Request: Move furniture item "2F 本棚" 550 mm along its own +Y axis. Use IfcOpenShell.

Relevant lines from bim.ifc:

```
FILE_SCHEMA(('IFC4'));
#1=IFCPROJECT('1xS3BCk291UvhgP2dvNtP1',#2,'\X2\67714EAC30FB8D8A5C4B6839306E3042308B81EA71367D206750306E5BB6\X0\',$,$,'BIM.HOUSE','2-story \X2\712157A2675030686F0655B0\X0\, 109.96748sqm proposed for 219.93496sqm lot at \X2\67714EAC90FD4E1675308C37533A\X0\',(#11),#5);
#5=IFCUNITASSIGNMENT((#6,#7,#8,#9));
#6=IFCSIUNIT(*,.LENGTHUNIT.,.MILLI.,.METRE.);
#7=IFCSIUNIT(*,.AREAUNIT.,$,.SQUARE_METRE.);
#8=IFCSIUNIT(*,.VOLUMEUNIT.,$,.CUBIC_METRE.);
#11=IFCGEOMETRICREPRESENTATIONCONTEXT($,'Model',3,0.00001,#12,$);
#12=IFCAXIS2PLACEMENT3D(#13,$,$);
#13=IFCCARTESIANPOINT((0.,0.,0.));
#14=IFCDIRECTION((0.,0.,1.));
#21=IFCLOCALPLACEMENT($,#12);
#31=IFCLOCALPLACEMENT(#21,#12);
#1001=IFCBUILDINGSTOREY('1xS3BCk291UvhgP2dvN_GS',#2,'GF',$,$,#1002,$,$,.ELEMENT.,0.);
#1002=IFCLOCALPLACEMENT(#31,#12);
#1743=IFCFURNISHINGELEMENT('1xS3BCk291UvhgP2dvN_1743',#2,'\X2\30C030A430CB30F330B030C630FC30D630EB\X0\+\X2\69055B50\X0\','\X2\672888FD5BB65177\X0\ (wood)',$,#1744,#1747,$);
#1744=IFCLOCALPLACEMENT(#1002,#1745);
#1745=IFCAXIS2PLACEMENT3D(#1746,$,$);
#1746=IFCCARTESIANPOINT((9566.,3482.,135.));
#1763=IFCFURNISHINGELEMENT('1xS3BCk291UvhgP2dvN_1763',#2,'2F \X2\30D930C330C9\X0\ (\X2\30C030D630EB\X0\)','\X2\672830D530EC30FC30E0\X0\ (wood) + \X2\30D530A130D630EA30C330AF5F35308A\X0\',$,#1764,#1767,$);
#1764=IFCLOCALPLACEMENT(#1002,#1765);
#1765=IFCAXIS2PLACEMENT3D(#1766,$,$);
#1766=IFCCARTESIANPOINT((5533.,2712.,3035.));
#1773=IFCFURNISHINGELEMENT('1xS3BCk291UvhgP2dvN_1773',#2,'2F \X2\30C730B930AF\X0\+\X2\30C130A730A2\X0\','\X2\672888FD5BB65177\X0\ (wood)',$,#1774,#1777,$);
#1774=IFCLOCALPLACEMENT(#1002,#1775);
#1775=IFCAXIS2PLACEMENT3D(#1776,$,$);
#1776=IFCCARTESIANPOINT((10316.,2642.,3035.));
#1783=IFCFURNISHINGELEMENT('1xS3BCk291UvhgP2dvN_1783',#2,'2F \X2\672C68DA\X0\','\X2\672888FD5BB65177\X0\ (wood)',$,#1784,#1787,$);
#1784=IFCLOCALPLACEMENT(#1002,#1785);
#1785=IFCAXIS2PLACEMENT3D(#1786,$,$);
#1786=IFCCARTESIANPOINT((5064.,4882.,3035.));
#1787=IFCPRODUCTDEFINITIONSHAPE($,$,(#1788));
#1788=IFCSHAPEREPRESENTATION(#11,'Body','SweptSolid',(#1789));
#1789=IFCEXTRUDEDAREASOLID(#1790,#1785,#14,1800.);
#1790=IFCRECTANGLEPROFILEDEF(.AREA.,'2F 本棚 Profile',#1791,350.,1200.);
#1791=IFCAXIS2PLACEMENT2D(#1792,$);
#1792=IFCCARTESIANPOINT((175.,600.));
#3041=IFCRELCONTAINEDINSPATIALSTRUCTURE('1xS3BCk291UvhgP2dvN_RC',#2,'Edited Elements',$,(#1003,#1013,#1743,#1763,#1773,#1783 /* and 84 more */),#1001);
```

```python
import ifcopenshell
import ifcopenshell.api.geometry
import ifcopenshell.util.placement

model = ifcopenshell.open("bim.ifc")

item = model.by_id(1783)
matrix = ifcopenshell.util.placement.get_local_placement(item.ObjectPlacement)
matrix[:3, 3] += matrix[:3, 1] * 550.0
ifcopenshell.api.geometry.edit_object_placement(model, product=item, matrix=matrix, is_si=False)

print(ifcopenshell.util.placement.get_local_placement(item.ObjectPlacement).round(3) + 0.0)

model.write("bim-out.ifc")
```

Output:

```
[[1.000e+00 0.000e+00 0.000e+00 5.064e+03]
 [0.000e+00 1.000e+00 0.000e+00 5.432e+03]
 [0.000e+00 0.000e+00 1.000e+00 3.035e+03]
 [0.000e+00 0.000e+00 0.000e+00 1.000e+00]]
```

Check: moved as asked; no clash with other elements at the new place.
